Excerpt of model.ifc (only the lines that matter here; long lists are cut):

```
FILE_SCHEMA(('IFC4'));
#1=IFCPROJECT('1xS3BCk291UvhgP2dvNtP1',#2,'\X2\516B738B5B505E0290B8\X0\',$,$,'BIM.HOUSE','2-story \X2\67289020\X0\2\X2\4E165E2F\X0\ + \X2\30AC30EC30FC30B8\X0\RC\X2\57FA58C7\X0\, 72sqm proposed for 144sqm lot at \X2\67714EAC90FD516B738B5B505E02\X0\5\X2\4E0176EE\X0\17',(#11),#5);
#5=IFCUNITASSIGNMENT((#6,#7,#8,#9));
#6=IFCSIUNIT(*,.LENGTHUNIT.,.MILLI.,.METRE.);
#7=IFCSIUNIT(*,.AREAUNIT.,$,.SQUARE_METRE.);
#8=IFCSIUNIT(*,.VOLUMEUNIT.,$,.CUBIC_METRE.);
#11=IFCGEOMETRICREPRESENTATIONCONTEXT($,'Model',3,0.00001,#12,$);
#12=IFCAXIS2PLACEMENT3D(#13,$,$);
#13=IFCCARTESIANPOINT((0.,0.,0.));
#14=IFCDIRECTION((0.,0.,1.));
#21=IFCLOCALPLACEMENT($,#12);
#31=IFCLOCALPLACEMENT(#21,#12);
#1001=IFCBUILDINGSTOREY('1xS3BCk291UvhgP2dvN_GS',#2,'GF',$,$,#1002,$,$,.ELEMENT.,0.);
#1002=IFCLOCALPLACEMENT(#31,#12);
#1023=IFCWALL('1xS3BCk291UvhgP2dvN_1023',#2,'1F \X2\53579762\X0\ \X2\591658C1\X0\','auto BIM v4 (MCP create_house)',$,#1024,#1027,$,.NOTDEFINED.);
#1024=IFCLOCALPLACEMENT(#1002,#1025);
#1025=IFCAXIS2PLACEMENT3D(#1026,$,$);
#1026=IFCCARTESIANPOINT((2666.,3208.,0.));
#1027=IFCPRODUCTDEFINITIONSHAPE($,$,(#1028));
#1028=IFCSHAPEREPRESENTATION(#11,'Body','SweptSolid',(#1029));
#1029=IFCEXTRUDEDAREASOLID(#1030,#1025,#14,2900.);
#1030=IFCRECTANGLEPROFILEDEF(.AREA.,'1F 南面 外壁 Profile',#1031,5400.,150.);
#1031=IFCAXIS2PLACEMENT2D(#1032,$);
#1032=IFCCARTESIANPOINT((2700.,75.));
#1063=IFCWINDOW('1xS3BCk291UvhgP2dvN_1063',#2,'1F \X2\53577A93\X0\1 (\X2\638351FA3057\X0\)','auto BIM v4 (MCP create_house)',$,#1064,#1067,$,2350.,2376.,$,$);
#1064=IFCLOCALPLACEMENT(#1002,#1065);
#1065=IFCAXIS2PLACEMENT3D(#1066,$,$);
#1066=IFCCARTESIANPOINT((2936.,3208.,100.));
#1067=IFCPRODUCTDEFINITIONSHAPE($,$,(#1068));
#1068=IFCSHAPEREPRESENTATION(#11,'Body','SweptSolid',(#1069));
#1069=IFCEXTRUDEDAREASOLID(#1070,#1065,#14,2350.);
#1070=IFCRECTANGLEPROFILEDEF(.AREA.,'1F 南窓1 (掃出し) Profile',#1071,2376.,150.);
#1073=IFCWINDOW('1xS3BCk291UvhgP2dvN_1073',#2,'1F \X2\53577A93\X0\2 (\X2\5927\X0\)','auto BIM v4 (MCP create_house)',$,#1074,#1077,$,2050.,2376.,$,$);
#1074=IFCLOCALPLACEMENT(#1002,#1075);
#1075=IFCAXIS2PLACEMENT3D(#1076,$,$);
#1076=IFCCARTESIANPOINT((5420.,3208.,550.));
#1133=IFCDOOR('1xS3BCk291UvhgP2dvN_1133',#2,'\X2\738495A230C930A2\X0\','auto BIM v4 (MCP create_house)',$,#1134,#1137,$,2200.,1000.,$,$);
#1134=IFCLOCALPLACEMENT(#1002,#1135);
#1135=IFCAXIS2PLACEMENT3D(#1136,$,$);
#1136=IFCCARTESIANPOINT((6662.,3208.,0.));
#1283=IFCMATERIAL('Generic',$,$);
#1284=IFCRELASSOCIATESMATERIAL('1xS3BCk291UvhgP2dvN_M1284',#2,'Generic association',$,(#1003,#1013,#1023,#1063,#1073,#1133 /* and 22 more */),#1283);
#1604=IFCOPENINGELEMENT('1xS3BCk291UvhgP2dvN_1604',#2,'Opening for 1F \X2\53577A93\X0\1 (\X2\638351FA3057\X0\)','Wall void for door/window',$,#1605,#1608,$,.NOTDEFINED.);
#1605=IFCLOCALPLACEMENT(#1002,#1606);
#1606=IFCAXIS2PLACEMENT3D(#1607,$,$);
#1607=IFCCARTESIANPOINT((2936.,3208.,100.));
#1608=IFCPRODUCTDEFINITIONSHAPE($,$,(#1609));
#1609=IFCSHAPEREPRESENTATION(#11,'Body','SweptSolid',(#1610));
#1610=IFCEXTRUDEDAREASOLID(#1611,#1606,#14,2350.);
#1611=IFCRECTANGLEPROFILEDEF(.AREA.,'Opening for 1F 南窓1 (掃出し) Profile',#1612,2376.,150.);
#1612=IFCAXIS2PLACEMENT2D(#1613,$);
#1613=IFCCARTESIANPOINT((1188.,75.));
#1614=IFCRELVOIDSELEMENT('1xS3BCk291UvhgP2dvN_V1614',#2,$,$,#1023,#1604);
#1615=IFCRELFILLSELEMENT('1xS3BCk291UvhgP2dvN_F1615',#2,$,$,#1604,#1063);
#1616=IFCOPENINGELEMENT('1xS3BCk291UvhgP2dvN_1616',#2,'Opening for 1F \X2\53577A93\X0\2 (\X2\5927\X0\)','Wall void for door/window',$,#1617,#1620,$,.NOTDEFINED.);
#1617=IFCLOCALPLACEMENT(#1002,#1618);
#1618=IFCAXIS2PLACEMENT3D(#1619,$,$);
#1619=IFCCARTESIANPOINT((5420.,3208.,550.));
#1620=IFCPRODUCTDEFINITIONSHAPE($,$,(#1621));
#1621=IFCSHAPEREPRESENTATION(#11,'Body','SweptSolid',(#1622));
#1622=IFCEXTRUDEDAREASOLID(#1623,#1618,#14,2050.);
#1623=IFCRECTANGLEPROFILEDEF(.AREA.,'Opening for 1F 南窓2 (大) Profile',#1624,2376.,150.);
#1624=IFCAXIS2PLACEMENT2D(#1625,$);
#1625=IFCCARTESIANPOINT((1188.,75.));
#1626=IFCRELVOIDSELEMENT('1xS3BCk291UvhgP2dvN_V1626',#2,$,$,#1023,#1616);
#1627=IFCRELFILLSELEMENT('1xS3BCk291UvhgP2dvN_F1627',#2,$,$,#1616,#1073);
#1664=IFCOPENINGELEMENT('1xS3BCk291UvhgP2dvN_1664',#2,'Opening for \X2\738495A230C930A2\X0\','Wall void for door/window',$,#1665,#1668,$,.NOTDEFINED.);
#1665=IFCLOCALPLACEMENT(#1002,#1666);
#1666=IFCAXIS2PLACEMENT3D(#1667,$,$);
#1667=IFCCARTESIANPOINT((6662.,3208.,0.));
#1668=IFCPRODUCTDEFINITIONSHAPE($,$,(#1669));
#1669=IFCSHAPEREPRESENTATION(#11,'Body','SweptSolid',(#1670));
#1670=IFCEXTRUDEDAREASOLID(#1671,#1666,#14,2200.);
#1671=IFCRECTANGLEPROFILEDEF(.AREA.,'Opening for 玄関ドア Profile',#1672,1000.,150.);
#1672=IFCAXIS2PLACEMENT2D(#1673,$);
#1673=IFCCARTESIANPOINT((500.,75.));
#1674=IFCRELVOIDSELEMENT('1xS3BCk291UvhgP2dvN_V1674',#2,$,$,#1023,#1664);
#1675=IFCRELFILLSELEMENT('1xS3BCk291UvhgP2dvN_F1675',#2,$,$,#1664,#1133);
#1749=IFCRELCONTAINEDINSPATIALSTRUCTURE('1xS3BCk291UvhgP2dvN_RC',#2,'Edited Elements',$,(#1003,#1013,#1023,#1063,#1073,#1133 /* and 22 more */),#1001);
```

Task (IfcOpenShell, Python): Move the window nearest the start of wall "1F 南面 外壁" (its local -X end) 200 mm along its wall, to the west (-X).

```python
import ifcopenshell
import ifcopenshell.api.geometry
import ifcopenshell.util.placement
import ifcopenshell.util.unit

model = ifcopenshell.open("model.ifc")
unit_scale = ifcopenshell.util.unit.calculate_unit_scale(model)

window = model.by_id(1063)
opening = window.FillsVoids[0].RelatingOpeningElement
wall = opening.VoidsElements[0].RelatingBuildingElement

wall_matrix = ifcopenshell.util.placement.get_local_placement(wall.ObjectPlacement)
shift = wall_matrix[:3, 0] * -0.2 / unit_scale
before = ifcopenshell.util.placement.get_local_placement(window.ObjectPlacement)[:3, 3].copy()

# The window is not placed relative to its opening, so move both.
for product in (opening, window):
    matrix = ifcopenshell.util.placement.get_local_placement(product.ObjectPlacement)
    matrix[:3, 3] += shift
    ifcopenshell.api.geometry.edit_object_placement(model, product=product, matrix=matrix, is_si=False)

after = ifcopenshell.util.placement.get_local_placement(window.ObjectPlacement)[:3, 3]
print("window moved by", (after - before).round(3) + 0.0)

model.write("model-out.ifc")
```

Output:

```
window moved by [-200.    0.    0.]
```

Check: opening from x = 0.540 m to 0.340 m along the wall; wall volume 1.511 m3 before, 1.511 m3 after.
